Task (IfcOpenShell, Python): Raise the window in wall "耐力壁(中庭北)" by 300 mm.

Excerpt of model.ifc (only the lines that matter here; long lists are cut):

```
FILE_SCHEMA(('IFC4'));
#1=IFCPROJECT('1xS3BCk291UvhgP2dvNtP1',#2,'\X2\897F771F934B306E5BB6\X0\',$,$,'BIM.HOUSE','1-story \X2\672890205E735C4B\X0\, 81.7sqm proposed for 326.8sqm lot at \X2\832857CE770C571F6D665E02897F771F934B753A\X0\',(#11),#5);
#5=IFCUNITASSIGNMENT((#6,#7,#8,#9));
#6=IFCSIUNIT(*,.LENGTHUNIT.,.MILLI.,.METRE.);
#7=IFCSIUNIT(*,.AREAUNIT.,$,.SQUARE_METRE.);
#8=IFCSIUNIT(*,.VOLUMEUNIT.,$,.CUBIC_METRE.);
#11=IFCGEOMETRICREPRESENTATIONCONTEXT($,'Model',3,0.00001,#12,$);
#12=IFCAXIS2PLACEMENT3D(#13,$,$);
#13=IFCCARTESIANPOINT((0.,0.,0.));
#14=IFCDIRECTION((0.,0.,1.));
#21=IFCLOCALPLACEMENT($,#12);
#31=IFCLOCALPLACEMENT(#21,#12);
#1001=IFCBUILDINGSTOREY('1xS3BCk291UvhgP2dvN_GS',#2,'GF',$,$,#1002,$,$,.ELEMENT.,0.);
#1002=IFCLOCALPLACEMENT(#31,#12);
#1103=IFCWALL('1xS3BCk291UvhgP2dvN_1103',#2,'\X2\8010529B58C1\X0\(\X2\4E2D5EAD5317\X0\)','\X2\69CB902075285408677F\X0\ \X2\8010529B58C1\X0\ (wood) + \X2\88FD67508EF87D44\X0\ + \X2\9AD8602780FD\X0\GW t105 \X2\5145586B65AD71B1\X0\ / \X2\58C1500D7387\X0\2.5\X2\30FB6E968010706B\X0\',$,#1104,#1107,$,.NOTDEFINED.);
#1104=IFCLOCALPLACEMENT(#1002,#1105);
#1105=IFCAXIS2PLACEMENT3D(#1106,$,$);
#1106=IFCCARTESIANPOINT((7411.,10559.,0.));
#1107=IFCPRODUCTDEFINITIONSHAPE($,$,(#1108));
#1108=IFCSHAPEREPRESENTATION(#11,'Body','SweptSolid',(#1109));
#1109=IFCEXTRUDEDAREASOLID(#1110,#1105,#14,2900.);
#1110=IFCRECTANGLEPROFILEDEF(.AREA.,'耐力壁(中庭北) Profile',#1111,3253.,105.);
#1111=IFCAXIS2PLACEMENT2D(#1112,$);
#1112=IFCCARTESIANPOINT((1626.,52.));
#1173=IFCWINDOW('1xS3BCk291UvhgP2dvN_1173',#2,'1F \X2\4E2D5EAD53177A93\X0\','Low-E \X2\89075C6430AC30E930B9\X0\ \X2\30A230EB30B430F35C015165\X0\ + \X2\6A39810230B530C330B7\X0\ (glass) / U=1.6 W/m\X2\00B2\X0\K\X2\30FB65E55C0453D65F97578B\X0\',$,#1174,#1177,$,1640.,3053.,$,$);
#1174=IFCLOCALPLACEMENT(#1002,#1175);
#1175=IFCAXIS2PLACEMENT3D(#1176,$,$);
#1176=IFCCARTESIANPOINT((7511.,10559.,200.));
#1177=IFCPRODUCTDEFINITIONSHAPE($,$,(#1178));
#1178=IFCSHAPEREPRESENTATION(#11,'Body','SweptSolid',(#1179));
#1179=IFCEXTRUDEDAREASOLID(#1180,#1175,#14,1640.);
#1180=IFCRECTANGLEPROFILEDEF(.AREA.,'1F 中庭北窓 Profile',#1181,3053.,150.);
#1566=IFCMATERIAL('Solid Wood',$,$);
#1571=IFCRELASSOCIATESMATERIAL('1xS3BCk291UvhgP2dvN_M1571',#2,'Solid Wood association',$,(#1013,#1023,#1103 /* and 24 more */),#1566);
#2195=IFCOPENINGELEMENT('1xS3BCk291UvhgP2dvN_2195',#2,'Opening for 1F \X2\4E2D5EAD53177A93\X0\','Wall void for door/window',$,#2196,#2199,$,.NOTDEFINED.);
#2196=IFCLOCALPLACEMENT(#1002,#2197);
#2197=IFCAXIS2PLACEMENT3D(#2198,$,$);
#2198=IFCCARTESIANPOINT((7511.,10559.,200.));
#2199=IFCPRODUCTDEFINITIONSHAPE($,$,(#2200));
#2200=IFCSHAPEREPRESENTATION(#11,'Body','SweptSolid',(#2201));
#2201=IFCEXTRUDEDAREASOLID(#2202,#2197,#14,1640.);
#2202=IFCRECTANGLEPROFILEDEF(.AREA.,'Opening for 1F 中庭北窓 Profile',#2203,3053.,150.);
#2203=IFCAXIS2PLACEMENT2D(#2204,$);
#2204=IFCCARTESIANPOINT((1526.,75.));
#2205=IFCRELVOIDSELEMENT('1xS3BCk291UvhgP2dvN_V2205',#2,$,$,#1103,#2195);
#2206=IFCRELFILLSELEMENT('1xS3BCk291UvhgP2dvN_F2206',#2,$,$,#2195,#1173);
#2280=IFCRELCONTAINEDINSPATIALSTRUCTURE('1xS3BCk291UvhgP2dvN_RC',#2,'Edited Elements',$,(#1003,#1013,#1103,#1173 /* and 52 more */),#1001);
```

```python
import numpy as np
import ifcopenshell
import ifcopenshell.api.geometry
import ifcopenshell.util.placement
import ifcopenshell.util.unit

model = ifcopenshell.open("model.ifc")
unit_scale = ifcopenshell.util.unit.calculate_unit_scale(model)

window = model.by_guid("1xS3BCk291UvhgP2dvN_1173")
opening = window.FillsVoids[0].RelatingOpeningElement
dz = 0.3 / unit_scale

shift = np.array([0.0, 0.0, dz])
# The window is not placed relative to its opening, so move both.
for product in (opening, window):
    matrix = ifcopenshell.util.placement.get_local_placement(product.ObjectPlacement)
    matrix[:3, 3] += shift
    ifcopenshell.api.geometry.edit_object_placement(model, product=product, matrix=matrix, is_si=False)

print(f"moved by {dz * unit_scale:+.3f} m")

model.write("model-out.ifc")
```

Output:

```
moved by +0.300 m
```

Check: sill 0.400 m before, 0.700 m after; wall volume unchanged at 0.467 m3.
